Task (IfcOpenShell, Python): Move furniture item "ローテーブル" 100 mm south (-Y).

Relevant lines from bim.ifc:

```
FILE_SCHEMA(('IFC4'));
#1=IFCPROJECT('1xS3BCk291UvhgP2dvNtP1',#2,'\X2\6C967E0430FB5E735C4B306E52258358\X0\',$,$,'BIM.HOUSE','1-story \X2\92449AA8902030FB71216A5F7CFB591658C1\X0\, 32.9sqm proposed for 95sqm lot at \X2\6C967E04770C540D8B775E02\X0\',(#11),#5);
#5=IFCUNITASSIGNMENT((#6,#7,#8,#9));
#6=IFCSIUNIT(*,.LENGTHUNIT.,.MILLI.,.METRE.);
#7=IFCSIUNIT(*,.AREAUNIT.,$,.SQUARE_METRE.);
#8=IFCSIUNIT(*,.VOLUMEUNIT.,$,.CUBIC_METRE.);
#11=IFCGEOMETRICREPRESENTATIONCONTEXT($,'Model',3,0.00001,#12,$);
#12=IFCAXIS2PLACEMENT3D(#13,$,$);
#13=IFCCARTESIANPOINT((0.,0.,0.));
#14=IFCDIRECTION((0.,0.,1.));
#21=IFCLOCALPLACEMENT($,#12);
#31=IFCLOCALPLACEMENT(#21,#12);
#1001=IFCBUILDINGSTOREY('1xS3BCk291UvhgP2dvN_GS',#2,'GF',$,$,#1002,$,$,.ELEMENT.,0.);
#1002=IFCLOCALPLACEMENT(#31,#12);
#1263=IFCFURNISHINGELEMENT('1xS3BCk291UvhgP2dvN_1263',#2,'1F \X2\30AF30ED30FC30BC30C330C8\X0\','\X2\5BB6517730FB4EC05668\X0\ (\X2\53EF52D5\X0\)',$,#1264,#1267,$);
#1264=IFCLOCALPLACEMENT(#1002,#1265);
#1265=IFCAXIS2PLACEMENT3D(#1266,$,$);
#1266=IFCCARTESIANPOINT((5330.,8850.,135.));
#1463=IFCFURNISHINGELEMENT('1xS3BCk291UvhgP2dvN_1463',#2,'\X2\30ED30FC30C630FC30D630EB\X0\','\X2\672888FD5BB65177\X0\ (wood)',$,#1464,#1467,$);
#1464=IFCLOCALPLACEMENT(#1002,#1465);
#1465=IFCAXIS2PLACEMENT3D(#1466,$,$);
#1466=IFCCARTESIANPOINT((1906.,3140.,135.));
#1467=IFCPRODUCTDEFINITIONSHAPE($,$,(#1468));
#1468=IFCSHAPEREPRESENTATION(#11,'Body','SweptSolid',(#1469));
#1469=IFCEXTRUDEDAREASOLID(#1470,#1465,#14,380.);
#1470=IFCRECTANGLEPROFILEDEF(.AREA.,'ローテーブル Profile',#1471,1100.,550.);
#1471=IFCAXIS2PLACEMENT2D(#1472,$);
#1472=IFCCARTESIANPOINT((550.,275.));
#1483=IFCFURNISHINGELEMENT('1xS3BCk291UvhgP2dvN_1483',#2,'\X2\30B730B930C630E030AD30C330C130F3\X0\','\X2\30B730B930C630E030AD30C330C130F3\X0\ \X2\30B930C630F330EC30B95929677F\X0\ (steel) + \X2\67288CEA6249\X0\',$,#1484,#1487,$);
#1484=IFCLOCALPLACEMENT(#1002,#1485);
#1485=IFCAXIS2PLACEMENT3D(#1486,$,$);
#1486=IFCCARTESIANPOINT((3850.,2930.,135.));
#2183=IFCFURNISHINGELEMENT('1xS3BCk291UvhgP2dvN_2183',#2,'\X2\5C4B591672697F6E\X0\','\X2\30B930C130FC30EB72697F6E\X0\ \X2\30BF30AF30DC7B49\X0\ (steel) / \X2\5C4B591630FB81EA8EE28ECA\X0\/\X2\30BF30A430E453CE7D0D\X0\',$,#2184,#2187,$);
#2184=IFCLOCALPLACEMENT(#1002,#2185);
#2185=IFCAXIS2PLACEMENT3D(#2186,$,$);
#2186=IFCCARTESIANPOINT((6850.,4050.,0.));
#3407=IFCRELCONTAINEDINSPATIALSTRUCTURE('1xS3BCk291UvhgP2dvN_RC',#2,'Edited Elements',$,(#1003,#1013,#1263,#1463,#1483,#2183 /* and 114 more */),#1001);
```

```python
import ifcopenshell
import ifcopenshell.api.geometry
import ifcopenshell.util.placement

model = ifcopenshell.open("bim.ifc")

item = model.by_guid("1xS3BCk291UvhgP2dvN_1463")
matrix = ifcopenshell.util.placement.get_local_placement(item.ObjectPlacement)
matrix[1, 3] -= 100.0
ifcopenshell.api.geometry.edit_object_placement(model, product=item, matrix=matrix, is_si=False)

print(ifcopenshell.util.placement.get_local_placement(item.ObjectPlacement).round(3) + 0.0)

model.write("bim_edited.ifc")
```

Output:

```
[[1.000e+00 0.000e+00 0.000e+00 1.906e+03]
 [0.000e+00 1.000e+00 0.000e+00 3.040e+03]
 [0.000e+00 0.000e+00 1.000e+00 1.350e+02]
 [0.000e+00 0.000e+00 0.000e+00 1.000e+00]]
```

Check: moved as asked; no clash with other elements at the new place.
